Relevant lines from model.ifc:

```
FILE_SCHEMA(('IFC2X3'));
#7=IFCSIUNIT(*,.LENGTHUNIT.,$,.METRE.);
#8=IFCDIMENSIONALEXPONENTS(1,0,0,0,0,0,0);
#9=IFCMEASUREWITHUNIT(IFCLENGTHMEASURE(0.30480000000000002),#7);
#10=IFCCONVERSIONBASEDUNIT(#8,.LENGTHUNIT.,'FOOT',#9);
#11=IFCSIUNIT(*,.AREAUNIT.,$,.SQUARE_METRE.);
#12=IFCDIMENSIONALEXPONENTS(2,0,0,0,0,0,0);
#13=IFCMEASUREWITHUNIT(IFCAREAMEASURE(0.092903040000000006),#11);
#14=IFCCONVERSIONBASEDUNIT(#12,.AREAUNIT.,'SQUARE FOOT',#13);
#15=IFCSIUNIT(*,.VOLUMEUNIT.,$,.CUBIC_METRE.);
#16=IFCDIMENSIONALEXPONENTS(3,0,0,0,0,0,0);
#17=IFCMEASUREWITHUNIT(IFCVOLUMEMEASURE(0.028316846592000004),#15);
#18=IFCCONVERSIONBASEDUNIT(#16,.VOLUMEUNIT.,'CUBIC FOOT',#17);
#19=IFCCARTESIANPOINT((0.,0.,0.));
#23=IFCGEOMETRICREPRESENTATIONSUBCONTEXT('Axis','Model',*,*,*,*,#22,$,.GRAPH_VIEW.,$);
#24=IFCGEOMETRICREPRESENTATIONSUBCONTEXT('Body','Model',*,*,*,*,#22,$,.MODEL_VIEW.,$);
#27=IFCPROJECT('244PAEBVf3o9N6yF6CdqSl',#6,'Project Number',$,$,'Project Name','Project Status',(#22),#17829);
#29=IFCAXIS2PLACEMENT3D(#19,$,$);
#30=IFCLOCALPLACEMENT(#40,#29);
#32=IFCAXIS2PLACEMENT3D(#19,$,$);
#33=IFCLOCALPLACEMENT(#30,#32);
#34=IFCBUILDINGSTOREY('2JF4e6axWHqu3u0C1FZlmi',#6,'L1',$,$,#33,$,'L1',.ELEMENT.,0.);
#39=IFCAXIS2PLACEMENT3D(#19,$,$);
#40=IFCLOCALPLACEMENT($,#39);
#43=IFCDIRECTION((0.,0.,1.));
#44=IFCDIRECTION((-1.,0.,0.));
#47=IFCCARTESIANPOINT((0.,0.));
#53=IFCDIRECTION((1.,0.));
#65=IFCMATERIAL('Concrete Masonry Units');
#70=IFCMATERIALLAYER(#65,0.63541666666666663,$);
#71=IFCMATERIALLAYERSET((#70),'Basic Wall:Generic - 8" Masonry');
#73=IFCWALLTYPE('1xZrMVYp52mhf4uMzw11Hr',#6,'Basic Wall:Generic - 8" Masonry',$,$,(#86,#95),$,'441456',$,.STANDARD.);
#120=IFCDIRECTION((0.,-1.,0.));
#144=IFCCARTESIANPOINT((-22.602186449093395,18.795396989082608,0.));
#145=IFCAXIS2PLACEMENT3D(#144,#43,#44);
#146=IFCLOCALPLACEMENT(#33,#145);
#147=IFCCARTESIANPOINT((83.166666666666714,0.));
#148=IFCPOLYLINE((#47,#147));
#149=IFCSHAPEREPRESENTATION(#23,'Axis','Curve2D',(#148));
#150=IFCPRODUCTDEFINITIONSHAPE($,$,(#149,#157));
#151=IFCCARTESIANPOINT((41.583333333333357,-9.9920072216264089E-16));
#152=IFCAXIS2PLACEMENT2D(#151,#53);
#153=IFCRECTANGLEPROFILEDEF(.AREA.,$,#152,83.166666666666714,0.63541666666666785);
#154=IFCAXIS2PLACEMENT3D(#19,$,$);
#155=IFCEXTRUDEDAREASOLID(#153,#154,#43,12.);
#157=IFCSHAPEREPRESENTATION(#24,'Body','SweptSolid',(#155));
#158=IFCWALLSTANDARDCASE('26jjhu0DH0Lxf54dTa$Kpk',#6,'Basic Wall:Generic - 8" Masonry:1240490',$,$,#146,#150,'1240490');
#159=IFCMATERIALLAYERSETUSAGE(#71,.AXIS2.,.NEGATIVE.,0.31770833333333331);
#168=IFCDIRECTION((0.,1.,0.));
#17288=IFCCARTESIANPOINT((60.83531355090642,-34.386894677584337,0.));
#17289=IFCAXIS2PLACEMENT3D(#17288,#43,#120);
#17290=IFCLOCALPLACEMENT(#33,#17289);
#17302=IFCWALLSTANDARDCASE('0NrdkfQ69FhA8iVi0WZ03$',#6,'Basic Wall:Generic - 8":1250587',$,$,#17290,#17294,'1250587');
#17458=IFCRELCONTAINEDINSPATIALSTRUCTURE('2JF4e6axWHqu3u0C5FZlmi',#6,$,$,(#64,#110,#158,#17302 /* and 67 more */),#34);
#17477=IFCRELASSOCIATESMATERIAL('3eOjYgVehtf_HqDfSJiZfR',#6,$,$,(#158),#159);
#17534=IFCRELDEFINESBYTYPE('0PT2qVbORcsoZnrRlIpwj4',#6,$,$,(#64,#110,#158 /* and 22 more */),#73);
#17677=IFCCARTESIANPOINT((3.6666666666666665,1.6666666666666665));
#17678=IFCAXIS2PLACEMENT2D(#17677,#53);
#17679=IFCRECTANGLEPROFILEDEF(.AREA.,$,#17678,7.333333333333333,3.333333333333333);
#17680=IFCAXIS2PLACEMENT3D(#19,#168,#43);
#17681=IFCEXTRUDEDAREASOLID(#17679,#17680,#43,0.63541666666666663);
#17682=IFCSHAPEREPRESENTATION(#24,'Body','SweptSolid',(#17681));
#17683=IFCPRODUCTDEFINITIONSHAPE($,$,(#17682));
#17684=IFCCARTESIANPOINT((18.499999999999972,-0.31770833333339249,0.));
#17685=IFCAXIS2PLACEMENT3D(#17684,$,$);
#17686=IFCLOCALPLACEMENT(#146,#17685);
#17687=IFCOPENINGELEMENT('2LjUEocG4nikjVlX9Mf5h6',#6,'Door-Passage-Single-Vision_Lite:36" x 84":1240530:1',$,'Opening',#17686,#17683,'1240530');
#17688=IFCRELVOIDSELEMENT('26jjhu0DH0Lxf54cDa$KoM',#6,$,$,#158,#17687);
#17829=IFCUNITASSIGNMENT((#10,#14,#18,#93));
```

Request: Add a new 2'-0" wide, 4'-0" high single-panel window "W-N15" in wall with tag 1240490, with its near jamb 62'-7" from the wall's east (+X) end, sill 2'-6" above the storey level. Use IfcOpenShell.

```python
import numpy as np
import ifcopenshell
import ifcopenshell.api.feature
import ifcopenshell.api.geometry
import ifcopenshell.api.root
import ifcopenshell.api.spatial
import ifcopenshell.api.type
import ifcopenshell.geom
import ifcopenshell.util.element
import ifcopenshell.util.placement
import ifcopenshell.util.representation
import ifcopenshell.util.shape
import ifcopenshell.util.unit

model = ifcopenshell.open("model.ifc")
unit_scale = ifcopenshell.util.unit.calculate_unit_scale(model)
settings = ifcopenshell.geom.settings()


def volume(element):
    """Net volume in cubic metres, openings subtracted."""
    shape = ifcopenshell.geom.create_shape(settings, element)
    return ifcopenshell.util.shape.get_volume(shape.geometry)


wall = model.by_id(158)
storey = ifcopenshell.util.element.get_container(wall, ifc_class="IfcBuildingStorey")
context = ifcopenshell.util.representation.get_context(model, "Model", "Body", "MODEL_VIEW")
before = volume(wall)

width, height, from_end, sill = 0.6096, 1.2192, 19.0754, 0.762  # metres

# The wall runs along its own X axis, and the end named is its -X end.
wall_shape = ifcopenshell.geom.create_shape(settings, wall)
x, y, z = ifcopenshell.util.shape.get_vertices(wall_shape.geometry).T
start = x.min() + from_end
face, thickness = float(y.min()), float(y.max() - y.min())
wall_matrix = ifcopenshell.util.placement.get_local_placement(wall.ObjectPlacement)
level = ifcopenshell.util.placement.get_local_placement(storey.ObjectPlacement)[2, 3]


def in_wall(x, y):
    """Placement at x, y metres in the wall's axes, at sill height."""
    matrix = wall_matrix.copy()
    matrix[:, 3] = wall_matrix @ np.array([x / unit_scale, y / unit_scale, 0.0, 1.0])
    matrix[2, 3] = level + sill / unit_scale
    return matrix


# Opening: a box that overshoots both wall faces by 50 mm.
opening = ifcopenshell.api.root.create_entity(model, ifc_class="IfcOpeningElement")
box = ifcopenshell.api.geometry.add_wall_representation(
    model, context=context, length=width, height=height, thickness=thickness + 0.1
)
ifcopenshell.api.geometry.assign_representation(model, product=opening, representation=box)
ifcopenshell.api.geometry.edit_object_placement(model, product=opening, matrix=in_wall(start, face - 0.05), is_si=False)
ifcopenshell.api.feature.add_feature(model, feature=opening, element=wall)

window = ifcopenshell.api.root.create_entity(model, ifc_class="IfcWindow", name="W-N15")
window.OverallWidth, window.OverallHeight = width / unit_scale, height / unit_scale
body = ifcopenshell.api.geometry.add_window_representation(
    model,
    context=context,
    overall_width=window.OverallWidth,
    overall_height=window.OverallHeight,
    partition_type="SINGLE_PANEL",
)
ifcopenshell.api.geometry.assign_representation(model, product=window, representation=body)
ifcopenshell.api.spatial.assign_container(model, products=[window], relating_structure=storey)
fills = ifcopenshell.api.feature.add_filling(model, opening=opening, element=window)
fills.OwnerHistory = window.OwnerHistory  # required in IFC2X3

# IFC2X3 keeps the operation on the window style.
style = ifcopenshell.api.root.create_entity(model, ifc_class="IfcWindowStyle", name="W-N15")
style.OperationType, style.ConstructionType = "SINGLE_PANEL", "NOTDEFINED"
style.ParameterTakesPrecedence = style.Sizeable = False
ifcopenshell.api.type.assign_type(model, related_objects=[window], relating_type=style)

# Centre the window in the wall's thickness.
ifcopenshell.api.geometry.edit_object_placement(model, product=window, matrix=in_wall(start, face), is_si=False)
window_shape = ifcopenshell.geom.create_shape(settings, window)
depth = ifcopenshell.util.shape.get_vertices(window_shape.geometry)[:, 1]
offset = face + thickness / 2 - (depth.min() + depth.max()) / 2
ifcopenshell.api.geometry.edit_object_placement(model, product=window, matrix=in_wall(start, offset), is_si=False)

after = volume(wall)

print(f"wall volume {before:.3f} -> {after:.3f} m3")

model.write("model-out.ifc")
```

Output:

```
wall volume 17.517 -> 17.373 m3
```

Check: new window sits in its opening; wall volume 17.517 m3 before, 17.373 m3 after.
